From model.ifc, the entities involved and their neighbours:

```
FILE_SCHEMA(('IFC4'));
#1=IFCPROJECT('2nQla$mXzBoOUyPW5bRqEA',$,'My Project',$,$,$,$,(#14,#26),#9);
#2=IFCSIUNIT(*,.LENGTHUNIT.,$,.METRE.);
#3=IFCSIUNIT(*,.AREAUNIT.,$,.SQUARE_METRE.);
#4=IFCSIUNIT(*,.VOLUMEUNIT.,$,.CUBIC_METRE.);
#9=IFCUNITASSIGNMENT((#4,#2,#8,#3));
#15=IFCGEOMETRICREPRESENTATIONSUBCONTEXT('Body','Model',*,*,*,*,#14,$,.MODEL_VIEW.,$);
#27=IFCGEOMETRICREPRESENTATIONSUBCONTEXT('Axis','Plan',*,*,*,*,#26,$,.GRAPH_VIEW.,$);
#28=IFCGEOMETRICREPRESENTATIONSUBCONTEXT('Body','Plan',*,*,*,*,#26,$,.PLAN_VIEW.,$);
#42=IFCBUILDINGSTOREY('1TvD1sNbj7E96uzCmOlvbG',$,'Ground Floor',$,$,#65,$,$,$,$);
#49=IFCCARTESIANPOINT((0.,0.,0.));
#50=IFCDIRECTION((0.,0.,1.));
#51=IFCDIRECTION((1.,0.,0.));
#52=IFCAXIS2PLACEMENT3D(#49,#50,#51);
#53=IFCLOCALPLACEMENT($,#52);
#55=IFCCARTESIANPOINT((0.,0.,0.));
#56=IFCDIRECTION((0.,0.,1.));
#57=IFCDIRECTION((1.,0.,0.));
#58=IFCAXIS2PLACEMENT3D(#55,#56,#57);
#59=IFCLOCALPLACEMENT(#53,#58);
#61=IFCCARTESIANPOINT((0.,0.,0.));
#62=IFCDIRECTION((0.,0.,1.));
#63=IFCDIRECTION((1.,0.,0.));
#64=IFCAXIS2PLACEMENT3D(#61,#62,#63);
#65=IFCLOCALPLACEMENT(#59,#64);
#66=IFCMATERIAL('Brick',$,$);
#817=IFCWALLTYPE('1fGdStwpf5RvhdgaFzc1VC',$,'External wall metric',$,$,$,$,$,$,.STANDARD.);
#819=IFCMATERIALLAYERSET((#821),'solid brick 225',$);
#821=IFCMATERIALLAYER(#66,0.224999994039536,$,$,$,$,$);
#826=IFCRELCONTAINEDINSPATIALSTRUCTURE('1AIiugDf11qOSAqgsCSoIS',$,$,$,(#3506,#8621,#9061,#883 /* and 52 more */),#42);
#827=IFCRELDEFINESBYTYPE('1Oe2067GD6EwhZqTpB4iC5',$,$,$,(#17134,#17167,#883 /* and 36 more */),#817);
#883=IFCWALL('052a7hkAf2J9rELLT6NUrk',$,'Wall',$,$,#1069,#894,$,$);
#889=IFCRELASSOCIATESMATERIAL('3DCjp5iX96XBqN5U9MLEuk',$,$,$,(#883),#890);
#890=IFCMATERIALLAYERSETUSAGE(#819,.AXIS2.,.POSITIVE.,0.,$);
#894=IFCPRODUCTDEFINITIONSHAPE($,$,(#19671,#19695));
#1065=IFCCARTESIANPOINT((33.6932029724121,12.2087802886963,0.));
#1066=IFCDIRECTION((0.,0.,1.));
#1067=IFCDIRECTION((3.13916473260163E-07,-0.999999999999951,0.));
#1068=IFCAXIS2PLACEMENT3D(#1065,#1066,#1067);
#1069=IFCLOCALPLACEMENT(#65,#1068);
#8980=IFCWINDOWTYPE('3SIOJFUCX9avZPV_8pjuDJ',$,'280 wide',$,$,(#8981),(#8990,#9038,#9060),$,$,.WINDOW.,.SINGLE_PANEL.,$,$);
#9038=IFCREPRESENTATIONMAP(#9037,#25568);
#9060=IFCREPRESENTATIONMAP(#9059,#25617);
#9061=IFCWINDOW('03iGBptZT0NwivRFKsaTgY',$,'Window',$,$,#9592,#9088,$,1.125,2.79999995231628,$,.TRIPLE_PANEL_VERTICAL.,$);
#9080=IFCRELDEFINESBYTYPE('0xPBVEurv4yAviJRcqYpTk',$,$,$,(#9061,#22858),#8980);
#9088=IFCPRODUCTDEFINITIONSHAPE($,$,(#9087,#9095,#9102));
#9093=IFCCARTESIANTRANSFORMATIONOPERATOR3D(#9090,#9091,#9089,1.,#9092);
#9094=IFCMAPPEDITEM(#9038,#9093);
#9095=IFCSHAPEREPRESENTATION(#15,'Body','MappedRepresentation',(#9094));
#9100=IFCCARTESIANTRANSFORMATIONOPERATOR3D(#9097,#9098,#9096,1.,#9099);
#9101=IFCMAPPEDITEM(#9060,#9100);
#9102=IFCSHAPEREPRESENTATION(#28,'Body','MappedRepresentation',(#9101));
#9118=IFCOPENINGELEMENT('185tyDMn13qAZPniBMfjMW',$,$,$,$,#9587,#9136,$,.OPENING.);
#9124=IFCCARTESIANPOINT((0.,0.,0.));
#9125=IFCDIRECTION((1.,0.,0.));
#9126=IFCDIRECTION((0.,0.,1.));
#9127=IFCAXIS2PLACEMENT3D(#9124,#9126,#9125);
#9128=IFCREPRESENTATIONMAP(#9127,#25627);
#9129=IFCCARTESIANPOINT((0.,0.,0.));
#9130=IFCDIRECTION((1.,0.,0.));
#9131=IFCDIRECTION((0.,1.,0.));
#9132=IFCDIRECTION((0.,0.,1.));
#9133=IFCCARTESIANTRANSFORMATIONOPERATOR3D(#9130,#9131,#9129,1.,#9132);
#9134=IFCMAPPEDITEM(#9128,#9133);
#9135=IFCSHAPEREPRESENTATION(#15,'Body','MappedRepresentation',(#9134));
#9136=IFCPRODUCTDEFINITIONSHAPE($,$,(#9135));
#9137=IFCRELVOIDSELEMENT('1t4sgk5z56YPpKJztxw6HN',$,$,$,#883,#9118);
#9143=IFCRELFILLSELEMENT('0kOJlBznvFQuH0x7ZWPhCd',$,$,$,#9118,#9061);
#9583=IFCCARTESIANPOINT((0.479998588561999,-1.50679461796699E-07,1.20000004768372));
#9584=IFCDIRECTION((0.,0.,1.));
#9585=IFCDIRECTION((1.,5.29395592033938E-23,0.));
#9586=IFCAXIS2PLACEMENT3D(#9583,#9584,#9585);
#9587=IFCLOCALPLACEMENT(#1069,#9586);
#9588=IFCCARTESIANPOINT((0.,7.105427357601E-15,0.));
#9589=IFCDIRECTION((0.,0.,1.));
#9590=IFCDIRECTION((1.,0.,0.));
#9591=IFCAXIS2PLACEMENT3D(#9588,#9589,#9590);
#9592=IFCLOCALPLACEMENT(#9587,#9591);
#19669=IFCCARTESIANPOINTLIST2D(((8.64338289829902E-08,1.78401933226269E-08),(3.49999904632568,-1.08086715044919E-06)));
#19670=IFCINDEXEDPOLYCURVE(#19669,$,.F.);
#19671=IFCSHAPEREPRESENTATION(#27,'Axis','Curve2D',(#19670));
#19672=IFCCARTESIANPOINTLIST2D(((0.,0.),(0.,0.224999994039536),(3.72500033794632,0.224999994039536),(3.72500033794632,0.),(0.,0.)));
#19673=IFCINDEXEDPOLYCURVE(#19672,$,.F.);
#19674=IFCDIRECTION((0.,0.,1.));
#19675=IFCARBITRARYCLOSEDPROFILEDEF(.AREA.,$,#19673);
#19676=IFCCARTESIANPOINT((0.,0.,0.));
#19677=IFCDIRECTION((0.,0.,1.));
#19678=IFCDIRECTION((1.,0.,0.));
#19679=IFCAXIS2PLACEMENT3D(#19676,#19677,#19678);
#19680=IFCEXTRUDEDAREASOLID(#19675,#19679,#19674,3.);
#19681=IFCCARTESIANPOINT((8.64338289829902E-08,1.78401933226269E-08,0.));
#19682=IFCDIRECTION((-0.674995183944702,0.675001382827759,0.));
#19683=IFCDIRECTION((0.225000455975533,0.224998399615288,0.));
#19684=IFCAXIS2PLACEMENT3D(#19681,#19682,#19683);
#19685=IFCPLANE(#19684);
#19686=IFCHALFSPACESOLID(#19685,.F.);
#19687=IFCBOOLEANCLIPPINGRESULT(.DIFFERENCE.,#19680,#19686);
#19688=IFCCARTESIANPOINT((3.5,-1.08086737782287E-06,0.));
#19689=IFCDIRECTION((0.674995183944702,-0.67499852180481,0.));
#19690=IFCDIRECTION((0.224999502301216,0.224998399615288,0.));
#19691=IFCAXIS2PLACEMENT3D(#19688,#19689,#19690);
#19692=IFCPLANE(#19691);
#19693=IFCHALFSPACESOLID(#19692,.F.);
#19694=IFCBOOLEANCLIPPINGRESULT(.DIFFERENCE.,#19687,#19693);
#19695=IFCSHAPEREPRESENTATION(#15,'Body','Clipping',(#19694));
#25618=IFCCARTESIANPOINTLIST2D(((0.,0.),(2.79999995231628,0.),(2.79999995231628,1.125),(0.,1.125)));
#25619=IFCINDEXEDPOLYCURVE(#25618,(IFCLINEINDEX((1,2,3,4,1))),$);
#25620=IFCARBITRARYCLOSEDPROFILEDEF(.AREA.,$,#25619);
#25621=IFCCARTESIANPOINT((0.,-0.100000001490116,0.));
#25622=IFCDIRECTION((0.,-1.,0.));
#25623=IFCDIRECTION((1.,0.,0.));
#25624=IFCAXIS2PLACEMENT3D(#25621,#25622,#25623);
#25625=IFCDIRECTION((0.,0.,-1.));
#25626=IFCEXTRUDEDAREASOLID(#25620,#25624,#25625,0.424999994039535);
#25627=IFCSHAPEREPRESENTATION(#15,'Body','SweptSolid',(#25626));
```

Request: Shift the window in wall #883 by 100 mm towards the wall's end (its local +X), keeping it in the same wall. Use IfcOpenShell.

```python
import ifcopenshell
import ifcopenshell.api.geometry
import ifcopenshell.util.placement

model = ifcopenshell.open("model.ifc")

window = model.by_guid("03iGBptZT0NwivRFKsaTgY")
opening = window.FillsVoids[0].RelatingOpeningElement
wall = opening.VoidsElements[0].RelatingBuildingElement

wall_matrix = ifcopenshell.util.placement.get_local_placement(wall.ObjectPlacement)
shift = wall_matrix[:3, 0] * 0.1
before = ifcopenshell.util.placement.get_local_placement(window.ObjectPlacement)[:3, 3].copy()

# The window is placed relative to its opening, so it follows when the opening moves.
matrix = ifcopenshell.util.placement.get_local_placement(opening.ObjectPlacement)
matrix[:3, 3] += shift
ifcopenshell.api.geometry.edit_object_placement(
    model, product=opening, matrix=matrix, is_si=False, should_transform_children=True
)

after = ifcopenshell.util.placement.get_local_placement(window.ObjectPlacement)[:3, 3]
print("window moved by", (after - before).round(3) + 0.0)

model.write("model_updated.ifc")
```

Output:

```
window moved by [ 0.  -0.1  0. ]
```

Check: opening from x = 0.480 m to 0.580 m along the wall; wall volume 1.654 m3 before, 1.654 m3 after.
